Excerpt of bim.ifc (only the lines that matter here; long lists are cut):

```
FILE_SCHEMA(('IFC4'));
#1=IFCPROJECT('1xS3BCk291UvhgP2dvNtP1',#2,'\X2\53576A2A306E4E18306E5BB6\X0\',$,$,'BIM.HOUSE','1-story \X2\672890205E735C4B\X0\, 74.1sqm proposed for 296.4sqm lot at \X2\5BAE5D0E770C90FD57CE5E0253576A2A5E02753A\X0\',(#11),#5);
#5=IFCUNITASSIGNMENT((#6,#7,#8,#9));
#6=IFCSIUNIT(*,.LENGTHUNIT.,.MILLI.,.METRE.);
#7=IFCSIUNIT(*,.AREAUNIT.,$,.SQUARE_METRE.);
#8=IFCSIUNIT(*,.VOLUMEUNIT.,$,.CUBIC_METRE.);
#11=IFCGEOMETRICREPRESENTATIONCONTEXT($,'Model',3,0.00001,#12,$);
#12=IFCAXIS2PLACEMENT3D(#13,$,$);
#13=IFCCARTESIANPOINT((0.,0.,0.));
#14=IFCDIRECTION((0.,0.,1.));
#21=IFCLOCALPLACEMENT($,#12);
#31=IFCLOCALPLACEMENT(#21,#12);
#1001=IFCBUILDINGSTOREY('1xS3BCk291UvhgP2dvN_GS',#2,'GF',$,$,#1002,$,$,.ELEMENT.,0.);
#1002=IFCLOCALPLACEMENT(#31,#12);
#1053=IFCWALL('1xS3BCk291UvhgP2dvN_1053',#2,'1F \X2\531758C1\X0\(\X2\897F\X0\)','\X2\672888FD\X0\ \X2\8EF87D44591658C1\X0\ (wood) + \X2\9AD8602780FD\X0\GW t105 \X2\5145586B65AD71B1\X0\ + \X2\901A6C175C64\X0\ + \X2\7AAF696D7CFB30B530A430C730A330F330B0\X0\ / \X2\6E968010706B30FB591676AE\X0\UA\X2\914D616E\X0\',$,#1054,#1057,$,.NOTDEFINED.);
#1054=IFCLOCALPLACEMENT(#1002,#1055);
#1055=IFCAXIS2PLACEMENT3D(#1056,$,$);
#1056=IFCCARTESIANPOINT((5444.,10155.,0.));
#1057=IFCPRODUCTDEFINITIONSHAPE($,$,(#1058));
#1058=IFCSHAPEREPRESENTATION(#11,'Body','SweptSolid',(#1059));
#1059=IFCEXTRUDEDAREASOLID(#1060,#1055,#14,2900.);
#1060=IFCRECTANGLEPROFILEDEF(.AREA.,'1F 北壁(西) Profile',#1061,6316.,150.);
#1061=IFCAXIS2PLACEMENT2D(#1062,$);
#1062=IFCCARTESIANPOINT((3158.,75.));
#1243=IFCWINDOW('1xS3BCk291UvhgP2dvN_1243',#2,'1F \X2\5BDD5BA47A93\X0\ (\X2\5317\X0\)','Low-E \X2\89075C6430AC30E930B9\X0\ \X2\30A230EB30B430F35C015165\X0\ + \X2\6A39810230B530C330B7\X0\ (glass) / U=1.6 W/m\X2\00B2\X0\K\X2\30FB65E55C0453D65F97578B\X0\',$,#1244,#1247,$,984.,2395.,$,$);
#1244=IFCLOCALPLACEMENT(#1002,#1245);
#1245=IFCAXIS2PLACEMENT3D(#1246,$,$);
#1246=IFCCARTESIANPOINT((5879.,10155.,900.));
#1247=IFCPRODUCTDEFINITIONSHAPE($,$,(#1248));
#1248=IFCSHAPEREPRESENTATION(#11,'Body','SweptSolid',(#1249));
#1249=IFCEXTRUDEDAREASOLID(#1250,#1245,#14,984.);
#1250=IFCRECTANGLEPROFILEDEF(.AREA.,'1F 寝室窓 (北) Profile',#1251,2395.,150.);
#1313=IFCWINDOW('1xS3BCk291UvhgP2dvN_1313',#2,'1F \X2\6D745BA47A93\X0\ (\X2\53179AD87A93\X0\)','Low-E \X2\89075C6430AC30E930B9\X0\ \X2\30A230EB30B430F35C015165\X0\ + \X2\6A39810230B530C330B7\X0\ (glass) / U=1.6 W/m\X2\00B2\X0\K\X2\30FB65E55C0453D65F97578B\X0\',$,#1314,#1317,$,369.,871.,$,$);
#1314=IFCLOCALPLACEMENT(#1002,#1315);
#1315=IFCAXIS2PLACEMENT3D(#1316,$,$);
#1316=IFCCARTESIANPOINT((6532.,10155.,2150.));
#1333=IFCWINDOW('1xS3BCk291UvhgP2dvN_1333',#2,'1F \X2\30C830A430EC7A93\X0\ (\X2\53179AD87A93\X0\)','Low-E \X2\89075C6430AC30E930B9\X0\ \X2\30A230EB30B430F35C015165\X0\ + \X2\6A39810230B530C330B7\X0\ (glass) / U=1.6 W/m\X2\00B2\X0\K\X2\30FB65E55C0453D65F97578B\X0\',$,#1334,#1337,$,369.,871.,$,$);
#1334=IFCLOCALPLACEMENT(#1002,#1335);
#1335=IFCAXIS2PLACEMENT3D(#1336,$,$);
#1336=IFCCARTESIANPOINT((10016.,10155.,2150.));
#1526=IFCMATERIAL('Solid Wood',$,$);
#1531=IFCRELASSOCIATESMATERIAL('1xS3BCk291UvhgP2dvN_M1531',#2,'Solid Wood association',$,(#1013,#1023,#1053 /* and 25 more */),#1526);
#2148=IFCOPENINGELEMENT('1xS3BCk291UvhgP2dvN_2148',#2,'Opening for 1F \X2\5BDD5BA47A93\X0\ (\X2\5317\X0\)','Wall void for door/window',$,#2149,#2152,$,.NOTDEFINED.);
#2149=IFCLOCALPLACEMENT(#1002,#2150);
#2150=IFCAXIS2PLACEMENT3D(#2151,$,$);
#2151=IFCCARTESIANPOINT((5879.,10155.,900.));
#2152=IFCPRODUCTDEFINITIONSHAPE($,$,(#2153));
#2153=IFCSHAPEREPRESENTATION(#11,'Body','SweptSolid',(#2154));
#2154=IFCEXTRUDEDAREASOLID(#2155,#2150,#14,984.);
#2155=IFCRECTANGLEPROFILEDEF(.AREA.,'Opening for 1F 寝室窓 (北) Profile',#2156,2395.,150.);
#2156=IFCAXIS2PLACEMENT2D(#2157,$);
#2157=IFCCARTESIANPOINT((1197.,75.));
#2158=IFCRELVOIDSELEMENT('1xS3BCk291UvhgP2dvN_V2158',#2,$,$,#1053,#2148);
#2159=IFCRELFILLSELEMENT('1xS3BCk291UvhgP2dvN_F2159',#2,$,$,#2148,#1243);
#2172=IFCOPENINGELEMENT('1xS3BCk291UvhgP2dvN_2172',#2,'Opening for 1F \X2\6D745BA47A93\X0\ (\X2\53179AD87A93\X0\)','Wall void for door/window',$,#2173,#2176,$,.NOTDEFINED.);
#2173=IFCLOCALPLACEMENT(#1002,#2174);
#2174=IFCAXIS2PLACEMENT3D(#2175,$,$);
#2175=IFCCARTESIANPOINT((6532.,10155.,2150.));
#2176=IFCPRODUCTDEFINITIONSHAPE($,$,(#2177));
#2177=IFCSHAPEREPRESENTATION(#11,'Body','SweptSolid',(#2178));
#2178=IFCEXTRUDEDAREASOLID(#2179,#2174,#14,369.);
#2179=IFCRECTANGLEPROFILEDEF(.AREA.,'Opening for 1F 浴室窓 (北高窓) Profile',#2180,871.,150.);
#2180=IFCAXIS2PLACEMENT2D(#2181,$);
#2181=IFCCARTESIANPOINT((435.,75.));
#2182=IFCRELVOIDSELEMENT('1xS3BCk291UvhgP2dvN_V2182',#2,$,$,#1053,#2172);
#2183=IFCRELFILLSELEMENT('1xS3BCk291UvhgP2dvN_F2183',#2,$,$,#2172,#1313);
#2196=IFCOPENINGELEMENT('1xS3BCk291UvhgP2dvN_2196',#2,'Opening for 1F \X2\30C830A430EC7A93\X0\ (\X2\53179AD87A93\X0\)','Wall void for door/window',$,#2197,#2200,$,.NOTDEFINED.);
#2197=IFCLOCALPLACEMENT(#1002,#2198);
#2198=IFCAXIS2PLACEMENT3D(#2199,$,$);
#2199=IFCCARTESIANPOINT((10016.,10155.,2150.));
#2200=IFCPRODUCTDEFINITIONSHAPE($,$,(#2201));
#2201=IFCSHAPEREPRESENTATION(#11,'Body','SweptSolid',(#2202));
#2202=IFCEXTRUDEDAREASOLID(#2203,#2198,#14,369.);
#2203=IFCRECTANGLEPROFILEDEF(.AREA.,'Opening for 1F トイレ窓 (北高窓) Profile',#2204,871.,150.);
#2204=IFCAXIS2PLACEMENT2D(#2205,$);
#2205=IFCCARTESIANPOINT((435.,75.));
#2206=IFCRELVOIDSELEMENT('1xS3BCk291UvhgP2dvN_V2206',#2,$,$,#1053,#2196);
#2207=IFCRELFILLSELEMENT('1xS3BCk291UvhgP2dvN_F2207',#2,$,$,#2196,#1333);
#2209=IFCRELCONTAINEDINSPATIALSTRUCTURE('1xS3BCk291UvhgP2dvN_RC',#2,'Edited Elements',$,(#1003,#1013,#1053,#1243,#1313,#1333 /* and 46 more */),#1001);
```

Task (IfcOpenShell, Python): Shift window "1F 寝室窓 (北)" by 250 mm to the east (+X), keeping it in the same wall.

```python
import ifcopenshell
import ifcopenshell.api.geometry
import ifcopenshell.util.placement

model = ifcopenshell.open("bim.ifc")

window = model.by_id(1243)
opening = window.FillsVoids[0].RelatingOpeningElement
wall = opening.VoidsElements[0].RelatingBuildingElement

wall_matrix = ifcopenshell.util.placement.get_local_placement(wall.ObjectPlacement)
shift = wall_matrix[:3, 0] * 250.0
before = ifcopenshell.util.placement.get_local_placement(window.ObjectPlacement)[:3, 3].copy()

# The window is not placed relative to its opening, so move both.
for product in (opening, window):
    matrix = ifcopenshell.util.placement.get_local_placement(product.ObjectPlacement)
    matrix[:3, 3] += shift
    ifcopenshell.api.geometry.edit_object_placement(model, product=product, matrix=matrix, is_si=False)

after = ifcopenshell.util.placement.get_local_placement(window.ObjectPlacement)[:3, 3]
print("window moved by", (after - before).round(3) + 0.0)

model.write("bim_v2.ifc")
```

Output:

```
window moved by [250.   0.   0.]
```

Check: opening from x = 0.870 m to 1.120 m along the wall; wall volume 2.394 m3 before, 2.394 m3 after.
